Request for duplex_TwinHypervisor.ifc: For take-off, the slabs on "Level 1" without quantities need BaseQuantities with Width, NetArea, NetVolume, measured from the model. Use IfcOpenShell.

First a look at what the model holds.

```python
import ifcopenshell
import ifcopenshell.util.element
import ifcopenshell.util.unit

model = ifcopenshell.open("duplex_TwinHypervisor.ifc")
print(model.schema)
for unit_type in ("LENGTHUNIT", "AREAUNIT", "VOLUMEUNIT"):
    print(unit_type, ifcopenshell.util.unit.calculate_unit_scale(model, unit_type))
storey = next(s for s in model.by_type("IfcBuildingStorey") if s.Name == "Level 1")
slabs = [e for e in ifcopenshell.util.element.get_decomposition(storey) if e.is_a("IfcSlab")]
for e in sorted(slabs, key=lambda e: e.id()):
    print(e.id(), e.is_a(), e.Name, list(ifcopenshell.util.element.get_psets(e, qtos_only=True)), sep=" | ")
```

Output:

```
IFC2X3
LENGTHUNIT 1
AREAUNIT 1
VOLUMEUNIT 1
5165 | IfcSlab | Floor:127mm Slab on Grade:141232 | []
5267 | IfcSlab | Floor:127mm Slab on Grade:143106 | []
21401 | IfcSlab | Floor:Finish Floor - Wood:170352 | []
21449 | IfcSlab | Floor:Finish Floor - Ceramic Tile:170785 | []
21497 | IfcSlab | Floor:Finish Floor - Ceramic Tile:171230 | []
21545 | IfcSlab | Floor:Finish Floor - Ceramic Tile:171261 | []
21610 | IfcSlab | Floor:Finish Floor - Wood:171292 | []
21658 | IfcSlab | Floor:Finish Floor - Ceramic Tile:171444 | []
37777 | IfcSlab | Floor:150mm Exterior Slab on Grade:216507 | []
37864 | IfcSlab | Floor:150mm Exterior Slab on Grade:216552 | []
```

```python
import ifcopenshell
import ifcopenshell.api.pset
import ifcopenshell.geom
import ifcopenshell.util.element
import ifcopenshell.util.shape
import ifcopenshell.util.unit

model = ifcopenshell.open("duplex_TwinHypervisor.ifc")
unit_scale = ifcopenshell.util.unit.calculate_unit_scale(model)
area_scale = ifcopenshell.util.unit.calculate_unit_scale(model, "AREAUNIT")
volume_scale = ifcopenshell.util.unit.calculate_unit_scale(model, "VOLUMEUNIT")
settings = ifcopenshell.geom.settings()

storey = next(s for s in model.by_type("IfcBuildingStorey") if s.Name == "Level 1")
slabs = [e for e in ifcopenshell.util.element.get_decomposition(storey) if e.is_a("IfcSlab")]

for e in sorted(slabs, key=lambda e: e.id()):
    if ifcopenshell.util.element.get_psets(e, qtos_only=True, should_inherit=False):
        continue
    # Geometry comes back in metres, in the element's own axes.
    shape = ifcopenshell.geom.create_shape(settings, e)
    values = {
        "Width": ifcopenshell.util.shape.get_z(shape.geometry) / unit_scale,
        "NetArea": ifcopenshell.util.shape.get_footprint_area(shape.geometry) / area_scale,
        "NetVolume": ifcopenshell.util.shape.get_volume(shape.geometry) / volume_scale,
    }
    qto = ifcopenshell.api.pset.add_qto(model, product=e, name="BaseQuantities")
    ifcopenshell.api.pset.edit_qto(model, qto=qto, properties=values)
    print(e.id(), {k: round(v, 3) for k, v in values.items()})

model.write("duplex_TwinHypervisor_rev.ifc")
```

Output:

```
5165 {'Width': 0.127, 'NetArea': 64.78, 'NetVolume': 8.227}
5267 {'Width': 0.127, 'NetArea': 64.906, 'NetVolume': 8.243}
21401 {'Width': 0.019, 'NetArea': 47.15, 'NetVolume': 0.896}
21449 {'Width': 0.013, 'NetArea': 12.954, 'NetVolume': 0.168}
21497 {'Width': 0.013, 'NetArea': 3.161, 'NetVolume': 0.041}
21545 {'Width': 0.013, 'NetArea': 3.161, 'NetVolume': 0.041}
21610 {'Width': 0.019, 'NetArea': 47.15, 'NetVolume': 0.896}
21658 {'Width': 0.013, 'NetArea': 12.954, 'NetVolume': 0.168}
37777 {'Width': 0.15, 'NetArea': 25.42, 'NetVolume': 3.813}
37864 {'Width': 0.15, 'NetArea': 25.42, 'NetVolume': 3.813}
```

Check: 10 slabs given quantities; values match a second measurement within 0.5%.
